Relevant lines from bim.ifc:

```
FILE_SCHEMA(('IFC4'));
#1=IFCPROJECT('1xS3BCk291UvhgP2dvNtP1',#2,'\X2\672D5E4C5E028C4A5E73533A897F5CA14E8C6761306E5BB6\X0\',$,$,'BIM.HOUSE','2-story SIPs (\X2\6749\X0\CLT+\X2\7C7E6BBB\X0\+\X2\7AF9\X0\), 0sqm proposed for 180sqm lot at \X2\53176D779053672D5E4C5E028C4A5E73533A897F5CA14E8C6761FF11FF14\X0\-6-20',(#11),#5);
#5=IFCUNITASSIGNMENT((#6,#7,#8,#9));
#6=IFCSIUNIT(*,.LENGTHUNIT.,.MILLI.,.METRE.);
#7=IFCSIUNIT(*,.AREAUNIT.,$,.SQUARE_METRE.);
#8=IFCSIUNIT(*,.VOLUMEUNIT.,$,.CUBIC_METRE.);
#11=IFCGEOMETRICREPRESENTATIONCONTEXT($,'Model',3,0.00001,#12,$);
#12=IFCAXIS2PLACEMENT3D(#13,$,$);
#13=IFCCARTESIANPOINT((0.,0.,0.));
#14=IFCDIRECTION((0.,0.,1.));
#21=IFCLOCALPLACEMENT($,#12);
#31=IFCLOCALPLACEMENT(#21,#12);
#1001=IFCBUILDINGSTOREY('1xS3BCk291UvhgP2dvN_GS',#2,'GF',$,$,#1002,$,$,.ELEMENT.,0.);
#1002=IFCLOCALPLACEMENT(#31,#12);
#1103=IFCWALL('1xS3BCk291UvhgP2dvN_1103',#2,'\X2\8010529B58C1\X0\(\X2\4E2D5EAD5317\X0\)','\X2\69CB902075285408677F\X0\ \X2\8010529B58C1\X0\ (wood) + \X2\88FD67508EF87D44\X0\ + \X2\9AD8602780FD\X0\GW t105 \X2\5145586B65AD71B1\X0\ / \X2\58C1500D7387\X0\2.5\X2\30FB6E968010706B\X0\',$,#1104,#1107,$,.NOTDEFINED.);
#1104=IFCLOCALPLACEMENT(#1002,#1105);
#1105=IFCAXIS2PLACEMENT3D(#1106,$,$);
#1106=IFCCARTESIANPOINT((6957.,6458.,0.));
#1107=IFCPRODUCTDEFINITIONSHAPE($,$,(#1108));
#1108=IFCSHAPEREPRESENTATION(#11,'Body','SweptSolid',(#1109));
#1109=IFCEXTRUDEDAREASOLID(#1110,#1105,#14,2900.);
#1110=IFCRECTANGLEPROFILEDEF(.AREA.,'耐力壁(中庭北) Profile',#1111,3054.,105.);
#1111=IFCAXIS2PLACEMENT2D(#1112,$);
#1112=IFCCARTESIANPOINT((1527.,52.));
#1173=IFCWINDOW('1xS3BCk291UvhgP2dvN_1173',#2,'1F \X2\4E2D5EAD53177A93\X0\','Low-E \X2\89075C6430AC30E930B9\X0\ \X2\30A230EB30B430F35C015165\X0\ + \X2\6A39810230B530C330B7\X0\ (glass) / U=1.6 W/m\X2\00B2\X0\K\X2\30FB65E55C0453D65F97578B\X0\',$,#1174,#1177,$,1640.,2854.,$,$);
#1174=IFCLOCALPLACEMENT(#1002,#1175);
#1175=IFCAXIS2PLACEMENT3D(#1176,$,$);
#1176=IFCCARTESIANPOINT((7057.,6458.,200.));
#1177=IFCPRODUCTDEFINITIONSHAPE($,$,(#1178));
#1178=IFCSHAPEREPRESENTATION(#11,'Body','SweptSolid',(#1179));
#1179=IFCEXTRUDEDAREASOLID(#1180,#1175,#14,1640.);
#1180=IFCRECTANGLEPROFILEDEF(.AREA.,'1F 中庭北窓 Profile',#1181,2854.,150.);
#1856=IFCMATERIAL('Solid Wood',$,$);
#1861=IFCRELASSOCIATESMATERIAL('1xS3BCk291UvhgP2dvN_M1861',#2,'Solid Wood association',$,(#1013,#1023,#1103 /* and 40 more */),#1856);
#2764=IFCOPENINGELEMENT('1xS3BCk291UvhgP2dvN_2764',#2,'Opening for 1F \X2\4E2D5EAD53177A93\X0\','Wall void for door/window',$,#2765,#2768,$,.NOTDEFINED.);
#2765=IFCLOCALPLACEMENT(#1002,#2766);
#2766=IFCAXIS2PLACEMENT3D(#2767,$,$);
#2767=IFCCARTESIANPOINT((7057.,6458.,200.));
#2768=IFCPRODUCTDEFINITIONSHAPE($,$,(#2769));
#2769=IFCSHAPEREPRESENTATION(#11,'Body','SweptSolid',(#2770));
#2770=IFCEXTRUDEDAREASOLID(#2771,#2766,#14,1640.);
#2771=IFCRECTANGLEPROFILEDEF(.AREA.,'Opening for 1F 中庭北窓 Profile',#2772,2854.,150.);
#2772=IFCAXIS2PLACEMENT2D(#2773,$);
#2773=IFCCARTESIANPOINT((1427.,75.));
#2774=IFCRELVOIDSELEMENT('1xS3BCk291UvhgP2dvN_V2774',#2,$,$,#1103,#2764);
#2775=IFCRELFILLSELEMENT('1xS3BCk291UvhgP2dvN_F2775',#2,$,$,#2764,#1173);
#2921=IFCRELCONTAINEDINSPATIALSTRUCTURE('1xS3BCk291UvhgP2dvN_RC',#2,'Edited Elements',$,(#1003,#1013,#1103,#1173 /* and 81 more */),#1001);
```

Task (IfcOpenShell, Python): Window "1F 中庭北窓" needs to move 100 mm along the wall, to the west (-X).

```python
import ifcopenshell
import ifcopenshell.api.geometry
import ifcopenshell.util.placement

model = ifcopenshell.open("bim.ifc")

window = model.by_id(1173)
opening = window.FillsVoids[0].RelatingOpeningElement
wall = opening.VoidsElements[0].RelatingBuildingElement

wall_matrix = ifcopenshell.util.placement.get_local_placement(wall.ObjectPlacement)
shift = wall_matrix[:3, 0] * -100.0
before = ifcopenshell.util.placement.get_local_placement(window.ObjectPlacement)[:3, 3].copy()

# The window is not placed relative to its opening, so move both.
for product in (opening, window):
    matrix = ifcopenshell.util.placement.get_local_placement(product.ObjectPlacement)
    matrix[:3, 3] += shift
    ifcopenshell.api.geometry.edit_object_placement(model, product=product, matrix=matrix, is_si=False)

after = ifcopenshell.util.placement.get_local_placement(window.ObjectPlacement)[:3, 3]
print("window moved by", (after - before).round(3) + 0.0)

model.write("bim_edited.ifc")
```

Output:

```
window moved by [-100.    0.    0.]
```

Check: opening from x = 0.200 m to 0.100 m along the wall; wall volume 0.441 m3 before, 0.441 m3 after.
